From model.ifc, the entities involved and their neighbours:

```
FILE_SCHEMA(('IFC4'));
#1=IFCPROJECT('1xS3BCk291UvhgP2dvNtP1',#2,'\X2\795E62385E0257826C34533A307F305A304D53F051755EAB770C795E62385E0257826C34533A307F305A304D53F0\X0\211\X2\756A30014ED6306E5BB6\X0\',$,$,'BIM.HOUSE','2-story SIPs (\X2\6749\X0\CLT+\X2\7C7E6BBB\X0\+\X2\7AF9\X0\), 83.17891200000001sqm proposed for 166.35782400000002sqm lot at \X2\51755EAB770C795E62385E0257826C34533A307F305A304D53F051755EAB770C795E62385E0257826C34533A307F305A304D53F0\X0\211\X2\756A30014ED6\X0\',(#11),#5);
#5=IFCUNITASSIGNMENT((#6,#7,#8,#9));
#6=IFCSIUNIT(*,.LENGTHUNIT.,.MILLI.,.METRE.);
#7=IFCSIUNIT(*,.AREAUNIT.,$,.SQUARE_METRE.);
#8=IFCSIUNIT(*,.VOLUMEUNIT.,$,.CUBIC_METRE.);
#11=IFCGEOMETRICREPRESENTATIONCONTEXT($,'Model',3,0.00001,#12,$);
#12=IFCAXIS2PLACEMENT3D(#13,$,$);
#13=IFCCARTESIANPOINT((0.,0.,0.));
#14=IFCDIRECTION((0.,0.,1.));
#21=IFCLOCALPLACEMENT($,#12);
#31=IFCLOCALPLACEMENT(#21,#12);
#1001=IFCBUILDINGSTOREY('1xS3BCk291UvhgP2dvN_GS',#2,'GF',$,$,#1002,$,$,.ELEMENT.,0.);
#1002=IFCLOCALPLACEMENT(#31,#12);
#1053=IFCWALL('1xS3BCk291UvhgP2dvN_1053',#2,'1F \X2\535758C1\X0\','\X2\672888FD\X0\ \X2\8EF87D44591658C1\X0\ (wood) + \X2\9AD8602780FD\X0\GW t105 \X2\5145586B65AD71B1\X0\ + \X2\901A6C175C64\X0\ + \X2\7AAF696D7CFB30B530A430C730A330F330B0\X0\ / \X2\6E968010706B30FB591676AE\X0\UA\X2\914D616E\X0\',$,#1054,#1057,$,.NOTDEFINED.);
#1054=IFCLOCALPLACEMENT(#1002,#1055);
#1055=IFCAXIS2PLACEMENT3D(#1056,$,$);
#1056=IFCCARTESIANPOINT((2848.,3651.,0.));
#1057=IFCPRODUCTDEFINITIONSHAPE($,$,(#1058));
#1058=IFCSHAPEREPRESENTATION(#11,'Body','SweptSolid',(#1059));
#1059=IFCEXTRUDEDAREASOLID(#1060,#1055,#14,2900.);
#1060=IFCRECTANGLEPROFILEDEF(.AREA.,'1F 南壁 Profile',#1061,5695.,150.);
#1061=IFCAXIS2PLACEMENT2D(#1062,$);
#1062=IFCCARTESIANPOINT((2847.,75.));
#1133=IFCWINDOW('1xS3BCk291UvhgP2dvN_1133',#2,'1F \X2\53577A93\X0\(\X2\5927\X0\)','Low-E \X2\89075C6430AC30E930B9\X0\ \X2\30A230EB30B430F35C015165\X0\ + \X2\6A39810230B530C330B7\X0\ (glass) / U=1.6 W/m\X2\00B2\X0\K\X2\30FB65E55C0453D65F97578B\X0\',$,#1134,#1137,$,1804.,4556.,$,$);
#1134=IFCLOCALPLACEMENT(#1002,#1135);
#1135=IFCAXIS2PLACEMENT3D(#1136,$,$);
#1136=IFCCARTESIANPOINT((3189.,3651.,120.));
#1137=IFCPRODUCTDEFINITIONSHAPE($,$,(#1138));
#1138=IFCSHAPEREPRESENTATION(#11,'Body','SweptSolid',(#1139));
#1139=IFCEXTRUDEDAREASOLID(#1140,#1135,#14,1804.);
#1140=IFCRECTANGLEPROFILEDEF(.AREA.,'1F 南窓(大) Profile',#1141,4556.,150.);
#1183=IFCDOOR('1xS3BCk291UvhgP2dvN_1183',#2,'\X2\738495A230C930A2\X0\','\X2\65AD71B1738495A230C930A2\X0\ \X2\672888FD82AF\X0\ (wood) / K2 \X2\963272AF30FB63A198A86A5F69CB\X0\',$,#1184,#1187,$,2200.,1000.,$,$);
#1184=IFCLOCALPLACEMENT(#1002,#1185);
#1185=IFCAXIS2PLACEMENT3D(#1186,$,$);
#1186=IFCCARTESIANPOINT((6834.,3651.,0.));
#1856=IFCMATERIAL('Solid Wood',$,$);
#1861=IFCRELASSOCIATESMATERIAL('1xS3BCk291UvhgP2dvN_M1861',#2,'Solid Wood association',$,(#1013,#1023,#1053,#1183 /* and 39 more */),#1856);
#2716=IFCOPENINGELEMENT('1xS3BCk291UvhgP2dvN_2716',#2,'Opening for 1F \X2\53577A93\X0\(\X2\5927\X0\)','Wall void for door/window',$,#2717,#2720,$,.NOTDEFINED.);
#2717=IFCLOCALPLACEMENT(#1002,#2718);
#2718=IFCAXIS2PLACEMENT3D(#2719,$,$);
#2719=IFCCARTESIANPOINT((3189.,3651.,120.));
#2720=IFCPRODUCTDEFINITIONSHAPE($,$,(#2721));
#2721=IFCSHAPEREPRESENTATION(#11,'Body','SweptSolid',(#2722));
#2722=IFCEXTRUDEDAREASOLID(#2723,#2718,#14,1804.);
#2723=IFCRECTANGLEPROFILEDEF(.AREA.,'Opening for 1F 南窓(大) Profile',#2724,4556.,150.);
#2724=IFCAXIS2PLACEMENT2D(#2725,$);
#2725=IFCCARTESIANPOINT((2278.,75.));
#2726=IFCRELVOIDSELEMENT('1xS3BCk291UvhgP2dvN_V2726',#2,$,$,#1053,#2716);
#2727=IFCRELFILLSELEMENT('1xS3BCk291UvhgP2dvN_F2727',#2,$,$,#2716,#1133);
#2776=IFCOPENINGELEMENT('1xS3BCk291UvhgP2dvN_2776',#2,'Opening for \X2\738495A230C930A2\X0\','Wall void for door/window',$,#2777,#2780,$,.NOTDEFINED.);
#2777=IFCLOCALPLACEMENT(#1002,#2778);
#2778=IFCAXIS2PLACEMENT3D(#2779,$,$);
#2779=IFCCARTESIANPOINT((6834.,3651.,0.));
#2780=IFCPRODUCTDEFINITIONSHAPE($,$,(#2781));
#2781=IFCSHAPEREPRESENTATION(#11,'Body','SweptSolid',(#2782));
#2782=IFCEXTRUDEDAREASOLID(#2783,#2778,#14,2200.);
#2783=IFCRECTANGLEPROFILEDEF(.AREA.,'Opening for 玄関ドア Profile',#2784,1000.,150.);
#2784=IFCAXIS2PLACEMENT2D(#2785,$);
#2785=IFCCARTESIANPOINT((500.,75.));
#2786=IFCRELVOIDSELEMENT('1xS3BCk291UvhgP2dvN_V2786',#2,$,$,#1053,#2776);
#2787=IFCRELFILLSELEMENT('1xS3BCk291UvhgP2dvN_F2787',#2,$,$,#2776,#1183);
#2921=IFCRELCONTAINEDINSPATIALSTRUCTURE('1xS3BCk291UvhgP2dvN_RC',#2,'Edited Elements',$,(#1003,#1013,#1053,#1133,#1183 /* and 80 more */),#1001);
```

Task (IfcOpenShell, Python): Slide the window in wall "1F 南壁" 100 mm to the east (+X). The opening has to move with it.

```python
import ifcopenshell
import ifcopenshell.api.geometry
import ifcopenshell.util.placement
import ifcopenshell.util.unit

model = ifcopenshell.open("model.ifc")
unit_scale = ifcopenshell.util.unit.calculate_unit_scale(model)

window = model.by_guid("1xS3BCk291UvhgP2dvN_1133")
opening = window.FillsVoids[0].RelatingOpeningElement
wall = opening.VoidsElements[0].RelatingBuildingElement

wall_matrix = ifcopenshell.util.placement.get_local_placement(wall.ObjectPlacement)
shift = wall_matrix[:3, 0] * 0.1 / unit_scale
before = ifcopenshell.util.placement.get_local_placement(window.ObjectPlacement)[:3, 3].copy()

# The window is not placed relative to its opening, so move both.
for product in (opening, window):
    matrix = ifcopenshell.util.placement.get_local_placement(product.ObjectPlacement)
    matrix[:3, 3] += shift
    ifcopenshell.api.geometry.edit_object_placement(model, product=product, matrix=matrix, is_si=False)

after = ifcopenshell.util.placement.get_local_placement(window.ObjectPlacement)[:3, 3]
print("window moved by", (after - before).round(3) + 0.0)

model.write("model_updated.ifc")
```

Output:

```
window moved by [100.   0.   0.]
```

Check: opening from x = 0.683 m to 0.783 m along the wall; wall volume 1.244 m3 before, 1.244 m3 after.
